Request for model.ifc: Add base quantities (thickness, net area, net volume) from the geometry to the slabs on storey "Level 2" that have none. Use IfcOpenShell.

First a look at what the model holds.

```python
import ifcopenshell
import ifcopenshell.util.element
import ifcopenshell.util.unit

model = ifcopenshell.open("model.ifc")
print(model.schema)
for unit_type in ("LENGTHUNIT", "AREAUNIT", "VOLUMEUNIT"):
    print(unit_type, ifcopenshell.util.unit.calculate_unit_scale(model, unit_type))
storey = next(s for s in model.by_type("IfcBuildingStorey") if s.Name == "Level 2")
slabs = [e for e in ifcopenshell.util.element.get_decomposition(storey) if e.is_a("IfcSlab")]
for e in sorted(slabs, key=lambda e: e.id()):
    print(e.id(), e.is_a(), e.Name, list(ifcopenshell.util.element.get_psets(e, qtos_only=True)), sep=" | ")
```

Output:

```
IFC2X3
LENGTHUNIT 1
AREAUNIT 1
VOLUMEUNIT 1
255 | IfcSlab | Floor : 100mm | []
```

```python
import ifcopenshell
import ifcopenshell.api.pset
import ifcopenshell.geom
import ifcopenshell.util.element
import ifcopenshell.util.shape
import ifcopenshell.util.unit

model = ifcopenshell.open("model.ifc")
unit_scale = ifcopenshell.util.unit.calculate_unit_scale(model)
area_scale = ifcopenshell.util.unit.calculate_unit_scale(model, "AREAUNIT")
volume_scale = ifcopenshell.util.unit.calculate_unit_scale(model, "VOLUMEUNIT")
settings = ifcopenshell.geom.settings()

storey = next(s for s in model.by_type("IfcBuildingStorey") if s.Name == "Level 2")
slabs = [e for e in ifcopenshell.util.element.get_decomposition(storey) if e.is_a("IfcSlab")]

for e in sorted(slabs, key=lambda e: e.id()):
    if ifcopenshell.util.element.get_psets(e, qtos_only=True, should_inherit=False):
        continue
    # Geometry comes back in metres, in the element's own axes.
    shape = ifcopenshell.geom.create_shape(settings, e)
    values = {
        "Width": ifcopenshell.util.shape.get_z(shape.geometry) / unit_scale,
        "NetArea": ifcopenshell.util.shape.get_footprint_area(shape.geometry) / area_scale,
        "NetVolume": ifcopenshell.util.shape.get_volume(shape.geometry) / volume_scale,
    }
    qto = ifcopenshell.api.pset.add_qto(model, product=e, name="BaseQuantities")
    ifcopenshell.api.pset.edit_qto(model, qto=qto, properties=values)
    print(e.id(), {k: round(v, 3) for k, v in values.items()})

model.write("model_v2.ifc")
```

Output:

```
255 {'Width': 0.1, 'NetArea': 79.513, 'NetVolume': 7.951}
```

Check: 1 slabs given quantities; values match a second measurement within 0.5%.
